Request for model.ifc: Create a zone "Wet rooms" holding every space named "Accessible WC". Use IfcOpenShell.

First a look at what the model holds.

```python
import ifcopenshell

model = ifcopenshell.open("model.ifc")
print(model.schema)
seen = {}
for space in model.by_type("IfcSpace"):
    seen[space.LongName] = seen.get(space.LongName, 0) + 1
for name, count in sorted(seen.items(), key=str):
    print(count, "x", name)
print("zones:", [z.Name for z in model.by_type("IfcZone")][:20])
```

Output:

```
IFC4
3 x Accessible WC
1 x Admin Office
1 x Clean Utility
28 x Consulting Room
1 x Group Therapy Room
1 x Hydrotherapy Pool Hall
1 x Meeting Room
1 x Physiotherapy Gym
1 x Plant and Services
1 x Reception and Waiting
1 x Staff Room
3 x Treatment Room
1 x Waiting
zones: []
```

```python
import ifcopenshell
import ifcopenshell.api.group
import ifcopenshell.api.root

model = ifcopenshell.open("model.ifc")

names = {"Accessible WC"}
spaces = [s for s in model.by_type("IfcSpace") if s.LongName in names]

zone = ifcopenshell.api.root.create_entity(model, ifc_class="IfcZone", name="Wet rooms")
ifcopenshell.api.group.assign_group(model, products=spaces, group=zone)
print(len(spaces), "spaces in", zone.Name)

model.write("model_rev.ifc")
```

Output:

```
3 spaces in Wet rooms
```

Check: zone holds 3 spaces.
